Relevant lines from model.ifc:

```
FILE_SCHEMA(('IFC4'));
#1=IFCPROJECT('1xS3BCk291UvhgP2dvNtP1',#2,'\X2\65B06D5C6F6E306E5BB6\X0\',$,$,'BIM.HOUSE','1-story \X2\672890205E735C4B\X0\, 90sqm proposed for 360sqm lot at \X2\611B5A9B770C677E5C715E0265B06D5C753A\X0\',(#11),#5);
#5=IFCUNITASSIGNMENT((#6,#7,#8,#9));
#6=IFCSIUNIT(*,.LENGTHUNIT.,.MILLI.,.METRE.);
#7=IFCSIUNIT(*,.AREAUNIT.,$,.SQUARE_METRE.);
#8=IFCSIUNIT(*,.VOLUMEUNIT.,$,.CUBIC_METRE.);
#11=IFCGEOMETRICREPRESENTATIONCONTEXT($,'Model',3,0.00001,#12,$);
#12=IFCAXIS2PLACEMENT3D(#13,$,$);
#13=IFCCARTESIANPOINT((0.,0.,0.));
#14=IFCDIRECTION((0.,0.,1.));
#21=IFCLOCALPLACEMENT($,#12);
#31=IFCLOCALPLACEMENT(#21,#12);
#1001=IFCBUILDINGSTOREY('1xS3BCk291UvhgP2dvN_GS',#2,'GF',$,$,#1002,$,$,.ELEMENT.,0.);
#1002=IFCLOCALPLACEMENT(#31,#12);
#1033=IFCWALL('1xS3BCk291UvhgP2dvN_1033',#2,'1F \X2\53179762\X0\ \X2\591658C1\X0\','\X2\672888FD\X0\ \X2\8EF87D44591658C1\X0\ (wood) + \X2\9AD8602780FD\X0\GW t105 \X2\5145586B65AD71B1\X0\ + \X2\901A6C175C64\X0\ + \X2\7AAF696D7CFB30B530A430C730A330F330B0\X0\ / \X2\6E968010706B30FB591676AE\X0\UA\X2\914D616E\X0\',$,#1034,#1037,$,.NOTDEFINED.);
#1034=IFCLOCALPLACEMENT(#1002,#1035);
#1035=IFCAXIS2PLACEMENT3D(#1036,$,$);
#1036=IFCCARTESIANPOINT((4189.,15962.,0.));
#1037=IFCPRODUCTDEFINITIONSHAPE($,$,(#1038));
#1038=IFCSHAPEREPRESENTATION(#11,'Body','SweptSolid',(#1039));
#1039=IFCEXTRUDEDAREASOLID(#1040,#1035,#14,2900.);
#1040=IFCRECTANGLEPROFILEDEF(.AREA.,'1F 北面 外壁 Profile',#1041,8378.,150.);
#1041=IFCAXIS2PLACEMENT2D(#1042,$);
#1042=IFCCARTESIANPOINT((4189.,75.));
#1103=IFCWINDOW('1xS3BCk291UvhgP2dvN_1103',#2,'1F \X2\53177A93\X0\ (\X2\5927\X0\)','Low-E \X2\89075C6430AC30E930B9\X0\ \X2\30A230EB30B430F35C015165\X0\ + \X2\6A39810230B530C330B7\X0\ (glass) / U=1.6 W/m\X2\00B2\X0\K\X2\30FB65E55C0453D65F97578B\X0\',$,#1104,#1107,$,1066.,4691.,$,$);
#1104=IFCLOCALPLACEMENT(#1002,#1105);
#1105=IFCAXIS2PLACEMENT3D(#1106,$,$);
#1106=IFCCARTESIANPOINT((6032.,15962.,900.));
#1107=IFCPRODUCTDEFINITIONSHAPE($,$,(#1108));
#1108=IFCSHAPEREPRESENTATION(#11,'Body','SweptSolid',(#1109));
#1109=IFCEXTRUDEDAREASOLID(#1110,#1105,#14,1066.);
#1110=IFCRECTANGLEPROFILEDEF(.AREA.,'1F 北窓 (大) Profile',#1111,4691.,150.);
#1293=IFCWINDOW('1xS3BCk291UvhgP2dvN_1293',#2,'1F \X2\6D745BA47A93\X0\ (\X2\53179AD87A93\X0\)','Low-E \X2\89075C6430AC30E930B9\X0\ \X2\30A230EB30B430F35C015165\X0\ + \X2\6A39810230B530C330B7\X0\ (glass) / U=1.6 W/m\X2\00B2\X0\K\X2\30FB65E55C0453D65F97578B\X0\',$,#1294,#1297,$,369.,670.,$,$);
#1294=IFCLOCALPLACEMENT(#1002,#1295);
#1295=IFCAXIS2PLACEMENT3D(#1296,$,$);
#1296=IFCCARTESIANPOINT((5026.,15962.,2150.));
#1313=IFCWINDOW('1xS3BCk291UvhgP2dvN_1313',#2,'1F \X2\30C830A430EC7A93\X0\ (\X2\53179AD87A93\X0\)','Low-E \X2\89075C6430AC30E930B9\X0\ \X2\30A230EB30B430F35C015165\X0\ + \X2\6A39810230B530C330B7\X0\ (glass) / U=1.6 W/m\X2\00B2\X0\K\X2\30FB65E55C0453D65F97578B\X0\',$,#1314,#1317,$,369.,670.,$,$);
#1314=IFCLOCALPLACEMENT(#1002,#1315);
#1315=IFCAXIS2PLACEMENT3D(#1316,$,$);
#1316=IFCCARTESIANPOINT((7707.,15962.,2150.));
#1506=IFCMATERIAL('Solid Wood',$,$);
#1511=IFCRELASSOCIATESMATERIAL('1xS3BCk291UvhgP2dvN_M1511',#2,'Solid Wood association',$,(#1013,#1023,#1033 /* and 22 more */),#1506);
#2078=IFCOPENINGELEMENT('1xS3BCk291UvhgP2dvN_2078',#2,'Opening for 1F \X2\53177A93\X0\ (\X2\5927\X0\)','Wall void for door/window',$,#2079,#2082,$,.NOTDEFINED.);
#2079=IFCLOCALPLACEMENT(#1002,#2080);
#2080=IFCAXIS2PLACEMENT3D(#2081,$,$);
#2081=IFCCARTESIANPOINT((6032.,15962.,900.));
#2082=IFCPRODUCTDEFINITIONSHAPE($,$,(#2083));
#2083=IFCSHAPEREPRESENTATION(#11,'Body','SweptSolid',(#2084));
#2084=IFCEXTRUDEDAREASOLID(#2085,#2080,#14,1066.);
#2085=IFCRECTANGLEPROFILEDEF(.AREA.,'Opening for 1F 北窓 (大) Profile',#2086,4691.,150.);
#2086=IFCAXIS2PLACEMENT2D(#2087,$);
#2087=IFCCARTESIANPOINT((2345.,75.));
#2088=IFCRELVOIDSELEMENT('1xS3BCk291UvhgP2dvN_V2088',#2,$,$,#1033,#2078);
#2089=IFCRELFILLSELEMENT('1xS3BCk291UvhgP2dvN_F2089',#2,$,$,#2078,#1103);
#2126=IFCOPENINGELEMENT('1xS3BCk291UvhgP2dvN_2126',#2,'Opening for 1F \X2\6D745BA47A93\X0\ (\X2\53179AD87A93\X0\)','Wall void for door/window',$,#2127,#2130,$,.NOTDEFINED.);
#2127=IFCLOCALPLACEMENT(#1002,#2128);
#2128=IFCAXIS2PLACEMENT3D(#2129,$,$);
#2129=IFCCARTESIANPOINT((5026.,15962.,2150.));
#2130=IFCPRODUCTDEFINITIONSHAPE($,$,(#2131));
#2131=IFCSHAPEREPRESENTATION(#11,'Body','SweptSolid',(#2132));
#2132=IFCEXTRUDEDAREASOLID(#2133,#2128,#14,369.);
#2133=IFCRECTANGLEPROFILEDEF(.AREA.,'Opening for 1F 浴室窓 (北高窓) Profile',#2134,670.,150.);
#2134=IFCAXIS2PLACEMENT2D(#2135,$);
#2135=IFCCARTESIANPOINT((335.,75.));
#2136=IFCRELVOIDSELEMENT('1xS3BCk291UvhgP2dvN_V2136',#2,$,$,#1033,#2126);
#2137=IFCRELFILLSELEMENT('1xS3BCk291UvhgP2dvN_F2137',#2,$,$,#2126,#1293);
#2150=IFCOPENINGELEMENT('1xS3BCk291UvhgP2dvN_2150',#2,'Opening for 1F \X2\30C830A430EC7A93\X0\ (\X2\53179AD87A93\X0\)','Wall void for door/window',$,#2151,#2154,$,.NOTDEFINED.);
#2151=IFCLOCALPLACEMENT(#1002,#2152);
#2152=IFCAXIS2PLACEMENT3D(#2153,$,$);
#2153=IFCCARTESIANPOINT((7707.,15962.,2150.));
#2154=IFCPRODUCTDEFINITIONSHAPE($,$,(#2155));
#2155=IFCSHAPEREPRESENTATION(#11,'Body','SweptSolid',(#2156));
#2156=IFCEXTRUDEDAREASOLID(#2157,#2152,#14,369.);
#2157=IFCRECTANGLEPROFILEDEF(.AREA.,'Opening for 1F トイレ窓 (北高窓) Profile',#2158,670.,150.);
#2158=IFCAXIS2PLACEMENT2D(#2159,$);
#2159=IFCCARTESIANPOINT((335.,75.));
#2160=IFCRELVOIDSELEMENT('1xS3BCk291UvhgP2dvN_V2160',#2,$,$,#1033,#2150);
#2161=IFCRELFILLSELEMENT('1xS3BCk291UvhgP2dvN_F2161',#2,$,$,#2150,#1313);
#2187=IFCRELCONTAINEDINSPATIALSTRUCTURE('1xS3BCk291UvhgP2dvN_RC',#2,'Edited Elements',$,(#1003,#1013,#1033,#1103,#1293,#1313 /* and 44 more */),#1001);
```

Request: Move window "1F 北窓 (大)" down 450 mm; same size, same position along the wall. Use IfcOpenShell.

```python
import numpy as np
import ifcopenshell
import ifcopenshell.api.geometry
import ifcopenshell.util.placement
import ifcopenshell.util.unit

model = ifcopenshell.open("model.ifc")
unit_scale = ifcopenshell.util.unit.calculate_unit_scale(model)

window = model.by_guid("1xS3BCk291UvhgP2dvN_1103")
opening = window.FillsVoids[0].RelatingOpeningElement
dz = -450.0

shift = np.array([0.0, 0.0, dz])
# The window is not placed relative to its opening, so move both.
for product in (opening, window):
    matrix = ifcopenshell.util.placement.get_local_placement(product.ObjectPlacement)
    matrix[:3, 3] += shift
    ifcopenshell.api.geometry.edit_object_placement(model, product=product, matrix=matrix, is_si=False)

print(f"moved by {dz * unit_scale:+.3f} m")

model.write("model-out.ifc")
```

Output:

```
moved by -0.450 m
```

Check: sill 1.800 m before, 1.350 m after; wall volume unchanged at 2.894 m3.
